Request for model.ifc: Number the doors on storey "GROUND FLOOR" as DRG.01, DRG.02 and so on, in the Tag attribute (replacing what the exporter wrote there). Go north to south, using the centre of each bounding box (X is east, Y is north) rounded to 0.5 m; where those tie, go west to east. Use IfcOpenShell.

First a look at what the model holds.

```python
import ifcopenshell
import ifcopenshell.util.element
import ifcopenshell.util.placement

model = ifcopenshell.open("model.ifc")
print(model.schema)
storey = next(s for s in model.by_type("IfcBuildingStorey") if s.Name == "GROUND FLOOR")
doors = [e for e in ifcopenshell.util.element.get_decomposition(storey) if e.is_a("IfcDoor")]
for e in sorted(doors, key=lambda e: e.id()):
    origin = ifcopenshell.util.placement.get_local_placement(e.ObjectPlacement)[:3, 3]
    print(e.id(), e.Tag, e.Name, origin.round(2) + 0.0, sep=" | ")
```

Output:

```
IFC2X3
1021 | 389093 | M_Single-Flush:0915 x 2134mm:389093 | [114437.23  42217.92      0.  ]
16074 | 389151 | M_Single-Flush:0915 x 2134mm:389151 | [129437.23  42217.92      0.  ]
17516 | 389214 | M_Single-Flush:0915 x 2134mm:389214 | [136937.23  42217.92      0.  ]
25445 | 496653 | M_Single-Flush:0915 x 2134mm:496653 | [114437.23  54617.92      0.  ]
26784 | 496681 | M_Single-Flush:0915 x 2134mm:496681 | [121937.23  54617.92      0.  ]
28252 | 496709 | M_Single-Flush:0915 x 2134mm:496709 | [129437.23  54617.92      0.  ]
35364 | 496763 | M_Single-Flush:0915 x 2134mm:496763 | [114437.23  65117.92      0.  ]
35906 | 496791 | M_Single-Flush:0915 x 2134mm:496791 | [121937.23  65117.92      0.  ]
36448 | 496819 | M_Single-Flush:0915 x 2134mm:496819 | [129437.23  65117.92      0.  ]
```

```python
import ifcopenshell
import ifcopenshell.geom
import ifcopenshell.util.element
import ifcopenshell.util.shape

model = ifcopenshell.open("model.ifc")
settings = ifcopenshell.geom.settings()
settings.set("use-world-coords", True)


def centre(element):
    shape = ifcopenshell.geom.create_shape(settings, element)
    return ifcopenshell.util.shape.get_bbox_centroid(shape.geometry)


storey = next(s for s in model.by_type("IfcBuildingStorey") if s.Name == "GROUND FLOOR")
doors = [e for e in ifcopenshell.util.element.get_decomposition(storey) if e.is_a("IfcDoor")]

# Insertion points can sit at a corner or the storey origin, so sort by the geometry (in metres).
centres = {e: centre(e) for e in doors}
doors.sort(key=lambda e: (-round(centres[e][1] / 0.5), centres[e][0]))

for i, e in enumerate(doors, start=1):
    number = f"DRG.{i:02d}"
    e.Tag = number
    print(e.id(), number)

model.write("model_updated.ifc")
```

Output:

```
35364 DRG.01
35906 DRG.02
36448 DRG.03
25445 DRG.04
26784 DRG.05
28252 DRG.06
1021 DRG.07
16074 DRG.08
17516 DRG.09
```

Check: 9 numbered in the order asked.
